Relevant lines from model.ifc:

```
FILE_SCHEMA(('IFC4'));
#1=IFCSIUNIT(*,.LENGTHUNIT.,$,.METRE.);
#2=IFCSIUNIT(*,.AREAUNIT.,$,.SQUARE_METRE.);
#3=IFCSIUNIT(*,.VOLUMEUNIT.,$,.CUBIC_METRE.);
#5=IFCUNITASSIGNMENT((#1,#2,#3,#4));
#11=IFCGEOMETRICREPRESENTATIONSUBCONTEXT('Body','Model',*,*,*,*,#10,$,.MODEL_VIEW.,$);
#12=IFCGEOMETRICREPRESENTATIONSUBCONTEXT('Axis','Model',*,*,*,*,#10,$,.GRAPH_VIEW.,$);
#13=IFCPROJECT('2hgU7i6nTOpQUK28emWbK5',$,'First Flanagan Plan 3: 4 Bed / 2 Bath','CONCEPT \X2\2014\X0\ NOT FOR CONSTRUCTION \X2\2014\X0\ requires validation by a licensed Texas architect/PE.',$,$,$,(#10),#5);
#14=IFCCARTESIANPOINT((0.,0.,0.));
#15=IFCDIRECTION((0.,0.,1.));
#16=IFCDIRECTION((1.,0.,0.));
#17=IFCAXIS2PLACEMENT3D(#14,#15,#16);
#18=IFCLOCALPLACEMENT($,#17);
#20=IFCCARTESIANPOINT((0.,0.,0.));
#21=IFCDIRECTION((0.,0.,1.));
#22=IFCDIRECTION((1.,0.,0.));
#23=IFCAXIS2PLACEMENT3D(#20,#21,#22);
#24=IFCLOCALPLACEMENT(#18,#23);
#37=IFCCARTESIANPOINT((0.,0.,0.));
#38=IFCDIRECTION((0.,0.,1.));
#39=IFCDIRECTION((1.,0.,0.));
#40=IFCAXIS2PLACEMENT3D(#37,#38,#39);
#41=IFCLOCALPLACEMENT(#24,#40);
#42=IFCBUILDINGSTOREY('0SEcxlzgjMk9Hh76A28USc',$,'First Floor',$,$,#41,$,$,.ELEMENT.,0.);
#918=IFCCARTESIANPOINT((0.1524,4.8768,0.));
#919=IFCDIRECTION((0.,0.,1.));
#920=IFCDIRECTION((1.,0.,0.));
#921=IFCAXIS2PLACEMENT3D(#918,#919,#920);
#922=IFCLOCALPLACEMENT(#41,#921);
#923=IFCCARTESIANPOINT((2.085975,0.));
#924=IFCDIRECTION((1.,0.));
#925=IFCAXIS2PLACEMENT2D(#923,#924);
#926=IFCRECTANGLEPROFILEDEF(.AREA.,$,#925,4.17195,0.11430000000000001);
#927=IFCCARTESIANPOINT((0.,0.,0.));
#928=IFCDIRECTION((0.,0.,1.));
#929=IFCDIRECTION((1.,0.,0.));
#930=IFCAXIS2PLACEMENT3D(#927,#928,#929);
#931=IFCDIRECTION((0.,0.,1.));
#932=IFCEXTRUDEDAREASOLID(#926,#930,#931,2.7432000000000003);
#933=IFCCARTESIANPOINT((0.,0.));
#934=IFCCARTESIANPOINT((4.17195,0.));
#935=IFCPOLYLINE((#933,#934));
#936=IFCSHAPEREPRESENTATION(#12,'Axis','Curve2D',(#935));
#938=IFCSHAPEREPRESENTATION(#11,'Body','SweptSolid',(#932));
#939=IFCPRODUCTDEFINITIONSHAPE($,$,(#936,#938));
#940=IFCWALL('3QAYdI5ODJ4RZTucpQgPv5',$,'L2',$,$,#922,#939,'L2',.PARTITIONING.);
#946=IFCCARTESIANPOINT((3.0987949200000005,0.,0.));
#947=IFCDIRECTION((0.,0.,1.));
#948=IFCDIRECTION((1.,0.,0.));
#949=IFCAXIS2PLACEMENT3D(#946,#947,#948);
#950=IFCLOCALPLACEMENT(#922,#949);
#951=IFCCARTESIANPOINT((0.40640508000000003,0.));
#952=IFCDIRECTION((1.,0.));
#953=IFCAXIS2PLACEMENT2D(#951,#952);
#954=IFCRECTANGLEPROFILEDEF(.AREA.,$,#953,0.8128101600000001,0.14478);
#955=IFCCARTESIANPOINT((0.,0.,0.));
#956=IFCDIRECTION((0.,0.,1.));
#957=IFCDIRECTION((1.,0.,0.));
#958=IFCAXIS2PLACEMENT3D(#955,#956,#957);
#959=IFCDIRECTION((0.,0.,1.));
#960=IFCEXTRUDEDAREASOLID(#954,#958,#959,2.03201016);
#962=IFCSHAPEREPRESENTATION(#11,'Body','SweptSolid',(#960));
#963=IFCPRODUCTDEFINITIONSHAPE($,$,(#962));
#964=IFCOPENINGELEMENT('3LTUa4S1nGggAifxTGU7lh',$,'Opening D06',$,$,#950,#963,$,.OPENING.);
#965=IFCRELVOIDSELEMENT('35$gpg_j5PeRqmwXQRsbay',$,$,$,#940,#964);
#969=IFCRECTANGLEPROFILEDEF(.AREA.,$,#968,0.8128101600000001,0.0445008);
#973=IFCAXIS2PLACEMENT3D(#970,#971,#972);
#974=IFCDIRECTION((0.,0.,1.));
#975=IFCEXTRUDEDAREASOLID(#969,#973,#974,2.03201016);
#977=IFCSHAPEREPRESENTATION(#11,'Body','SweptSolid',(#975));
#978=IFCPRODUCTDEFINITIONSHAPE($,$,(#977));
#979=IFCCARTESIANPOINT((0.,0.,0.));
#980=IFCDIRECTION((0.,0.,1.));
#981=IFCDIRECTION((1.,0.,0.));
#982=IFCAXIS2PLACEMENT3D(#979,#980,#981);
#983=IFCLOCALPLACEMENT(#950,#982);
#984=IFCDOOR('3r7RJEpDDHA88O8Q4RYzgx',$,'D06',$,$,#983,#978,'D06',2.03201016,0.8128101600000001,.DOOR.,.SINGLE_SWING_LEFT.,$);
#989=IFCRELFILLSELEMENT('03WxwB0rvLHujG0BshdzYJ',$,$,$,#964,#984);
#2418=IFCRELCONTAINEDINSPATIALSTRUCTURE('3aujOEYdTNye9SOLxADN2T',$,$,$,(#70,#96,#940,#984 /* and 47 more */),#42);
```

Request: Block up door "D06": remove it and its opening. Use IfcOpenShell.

```python
import ifcopenshell
import ifcopenshell.api.feature
import ifcopenshell.api.root
import ifcopenshell.geom
import ifcopenshell.util.shape

model = ifcopenshell.open("model.ifc")
settings = ifcopenshell.geom.settings()


def volume(element):
    """Net volume in cubic metres, openings subtracted."""
    shape = ifcopenshell.geom.create_shape(settings, element)
    return ifcopenshell.util.shape.get_volume(shape.geometry)


door = model.by_guid("3r7RJEpDDHA88O8Q4RYzgx")
opening = door.FillsVoids[0].RelatingOpeningElement
wall = opening.VoidsElements[0].RelatingBuildingElement
before = volume(wall)

ifcopenshell.api.root.remove_product(model, product=door)
ifcopenshell.api.feature.remove_feature(model, feature=opening)

after = volume(wall)

print(f"wall volume {before:.3f} -> {after:.3f} m3")

model.write("model_rev.ifc")
```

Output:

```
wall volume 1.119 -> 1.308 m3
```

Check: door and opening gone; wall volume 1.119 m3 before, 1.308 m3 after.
